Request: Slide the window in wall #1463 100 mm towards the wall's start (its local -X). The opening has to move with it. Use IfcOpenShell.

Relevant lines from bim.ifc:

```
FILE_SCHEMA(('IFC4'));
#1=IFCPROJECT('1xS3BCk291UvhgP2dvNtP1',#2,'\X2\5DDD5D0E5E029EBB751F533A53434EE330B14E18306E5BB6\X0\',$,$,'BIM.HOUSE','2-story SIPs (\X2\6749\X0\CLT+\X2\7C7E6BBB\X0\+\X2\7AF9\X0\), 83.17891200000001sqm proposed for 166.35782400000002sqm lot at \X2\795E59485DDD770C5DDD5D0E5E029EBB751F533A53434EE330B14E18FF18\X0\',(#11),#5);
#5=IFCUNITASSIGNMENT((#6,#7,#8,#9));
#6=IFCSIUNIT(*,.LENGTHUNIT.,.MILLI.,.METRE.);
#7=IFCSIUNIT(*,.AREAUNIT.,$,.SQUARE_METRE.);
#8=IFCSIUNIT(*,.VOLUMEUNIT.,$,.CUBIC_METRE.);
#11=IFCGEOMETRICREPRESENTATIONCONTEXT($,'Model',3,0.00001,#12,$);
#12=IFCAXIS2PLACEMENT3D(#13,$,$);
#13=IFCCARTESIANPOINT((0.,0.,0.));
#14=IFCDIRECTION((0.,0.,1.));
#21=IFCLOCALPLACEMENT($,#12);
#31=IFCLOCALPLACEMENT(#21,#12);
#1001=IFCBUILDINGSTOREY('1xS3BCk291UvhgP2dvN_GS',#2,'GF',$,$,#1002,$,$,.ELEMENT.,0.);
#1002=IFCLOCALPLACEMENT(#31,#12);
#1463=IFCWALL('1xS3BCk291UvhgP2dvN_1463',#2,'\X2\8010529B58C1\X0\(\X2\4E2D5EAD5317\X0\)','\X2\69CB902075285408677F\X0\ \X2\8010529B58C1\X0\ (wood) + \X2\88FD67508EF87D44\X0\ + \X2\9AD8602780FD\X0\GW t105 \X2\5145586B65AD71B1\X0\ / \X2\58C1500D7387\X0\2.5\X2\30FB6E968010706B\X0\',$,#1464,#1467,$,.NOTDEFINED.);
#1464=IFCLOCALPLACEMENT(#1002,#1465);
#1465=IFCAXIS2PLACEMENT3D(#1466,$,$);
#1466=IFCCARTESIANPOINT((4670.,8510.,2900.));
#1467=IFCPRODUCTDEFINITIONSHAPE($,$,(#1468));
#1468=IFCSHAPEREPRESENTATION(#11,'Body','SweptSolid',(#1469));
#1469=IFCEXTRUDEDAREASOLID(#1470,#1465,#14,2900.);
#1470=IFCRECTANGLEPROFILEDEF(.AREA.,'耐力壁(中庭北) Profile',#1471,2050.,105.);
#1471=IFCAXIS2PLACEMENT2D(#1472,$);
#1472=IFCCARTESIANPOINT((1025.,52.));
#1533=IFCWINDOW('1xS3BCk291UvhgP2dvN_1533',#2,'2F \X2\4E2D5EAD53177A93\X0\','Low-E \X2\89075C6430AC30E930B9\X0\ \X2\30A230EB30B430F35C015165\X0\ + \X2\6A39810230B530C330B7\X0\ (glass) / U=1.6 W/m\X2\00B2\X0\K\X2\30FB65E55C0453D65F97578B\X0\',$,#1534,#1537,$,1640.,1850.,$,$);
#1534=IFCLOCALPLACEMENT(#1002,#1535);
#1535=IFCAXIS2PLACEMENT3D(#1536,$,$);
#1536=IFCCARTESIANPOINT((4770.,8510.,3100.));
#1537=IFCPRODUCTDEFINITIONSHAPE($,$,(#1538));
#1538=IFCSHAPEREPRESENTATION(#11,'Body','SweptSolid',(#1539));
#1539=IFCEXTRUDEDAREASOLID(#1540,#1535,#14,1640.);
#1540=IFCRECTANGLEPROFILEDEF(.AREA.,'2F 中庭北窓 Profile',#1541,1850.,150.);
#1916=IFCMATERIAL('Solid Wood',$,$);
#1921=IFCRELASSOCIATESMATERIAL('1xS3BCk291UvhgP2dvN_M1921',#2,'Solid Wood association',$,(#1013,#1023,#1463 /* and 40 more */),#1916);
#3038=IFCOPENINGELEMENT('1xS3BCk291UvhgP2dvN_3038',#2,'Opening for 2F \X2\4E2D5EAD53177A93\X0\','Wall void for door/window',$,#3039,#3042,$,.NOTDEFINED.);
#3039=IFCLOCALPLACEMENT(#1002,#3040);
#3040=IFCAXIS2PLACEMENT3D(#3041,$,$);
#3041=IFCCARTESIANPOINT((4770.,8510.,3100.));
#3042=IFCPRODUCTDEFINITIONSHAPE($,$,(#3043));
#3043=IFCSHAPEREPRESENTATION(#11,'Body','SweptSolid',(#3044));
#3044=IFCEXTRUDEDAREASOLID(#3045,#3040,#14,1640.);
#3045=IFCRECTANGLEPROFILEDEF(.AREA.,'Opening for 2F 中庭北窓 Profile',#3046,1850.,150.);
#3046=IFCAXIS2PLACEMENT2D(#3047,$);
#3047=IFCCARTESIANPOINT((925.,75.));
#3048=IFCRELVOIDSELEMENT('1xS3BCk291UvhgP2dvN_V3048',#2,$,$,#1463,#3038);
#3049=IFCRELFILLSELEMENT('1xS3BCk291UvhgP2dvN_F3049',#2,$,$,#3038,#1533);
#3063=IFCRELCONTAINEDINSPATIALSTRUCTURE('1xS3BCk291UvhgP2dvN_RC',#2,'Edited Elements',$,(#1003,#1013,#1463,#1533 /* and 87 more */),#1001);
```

```python
import ifcopenshell
import ifcopenshell.api.geometry
import ifcopenshell.util.placement

model = ifcopenshell.open("bim.ifc")

window = model.by_guid("1xS3BCk291UvhgP2dvN_1533")
opening = window.FillsVoids[0].RelatingOpeningElement
wall = opening.VoidsElements[0].RelatingBuildingElement

wall_matrix = ifcopenshell.util.placement.get_local_placement(wall.ObjectPlacement)
shift = wall_matrix[:3, 0] * -100.0
before = ifcopenshell.util.placement.get_local_placement(window.ObjectPlacement)[:3, 3].copy()

# The window is not placed relative to its opening, so move both.
for product in (opening, window):
    matrix = ifcopenshell.util.placement.get_local_placement(product.ObjectPlacement)
    matrix[:3, 3] += shift
    ifcopenshell.api.geometry.edit_object_placement(model, product=product, matrix=matrix, is_si=False)

after = ifcopenshell.util.placement.get_local_placement(window.ObjectPlacement)[:3, 3]
print("window moved by", (after - before).round(3) + 0.0)

model.write("bim-out.ifc")
```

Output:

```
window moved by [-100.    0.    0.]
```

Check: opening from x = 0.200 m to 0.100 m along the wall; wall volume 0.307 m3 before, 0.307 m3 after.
